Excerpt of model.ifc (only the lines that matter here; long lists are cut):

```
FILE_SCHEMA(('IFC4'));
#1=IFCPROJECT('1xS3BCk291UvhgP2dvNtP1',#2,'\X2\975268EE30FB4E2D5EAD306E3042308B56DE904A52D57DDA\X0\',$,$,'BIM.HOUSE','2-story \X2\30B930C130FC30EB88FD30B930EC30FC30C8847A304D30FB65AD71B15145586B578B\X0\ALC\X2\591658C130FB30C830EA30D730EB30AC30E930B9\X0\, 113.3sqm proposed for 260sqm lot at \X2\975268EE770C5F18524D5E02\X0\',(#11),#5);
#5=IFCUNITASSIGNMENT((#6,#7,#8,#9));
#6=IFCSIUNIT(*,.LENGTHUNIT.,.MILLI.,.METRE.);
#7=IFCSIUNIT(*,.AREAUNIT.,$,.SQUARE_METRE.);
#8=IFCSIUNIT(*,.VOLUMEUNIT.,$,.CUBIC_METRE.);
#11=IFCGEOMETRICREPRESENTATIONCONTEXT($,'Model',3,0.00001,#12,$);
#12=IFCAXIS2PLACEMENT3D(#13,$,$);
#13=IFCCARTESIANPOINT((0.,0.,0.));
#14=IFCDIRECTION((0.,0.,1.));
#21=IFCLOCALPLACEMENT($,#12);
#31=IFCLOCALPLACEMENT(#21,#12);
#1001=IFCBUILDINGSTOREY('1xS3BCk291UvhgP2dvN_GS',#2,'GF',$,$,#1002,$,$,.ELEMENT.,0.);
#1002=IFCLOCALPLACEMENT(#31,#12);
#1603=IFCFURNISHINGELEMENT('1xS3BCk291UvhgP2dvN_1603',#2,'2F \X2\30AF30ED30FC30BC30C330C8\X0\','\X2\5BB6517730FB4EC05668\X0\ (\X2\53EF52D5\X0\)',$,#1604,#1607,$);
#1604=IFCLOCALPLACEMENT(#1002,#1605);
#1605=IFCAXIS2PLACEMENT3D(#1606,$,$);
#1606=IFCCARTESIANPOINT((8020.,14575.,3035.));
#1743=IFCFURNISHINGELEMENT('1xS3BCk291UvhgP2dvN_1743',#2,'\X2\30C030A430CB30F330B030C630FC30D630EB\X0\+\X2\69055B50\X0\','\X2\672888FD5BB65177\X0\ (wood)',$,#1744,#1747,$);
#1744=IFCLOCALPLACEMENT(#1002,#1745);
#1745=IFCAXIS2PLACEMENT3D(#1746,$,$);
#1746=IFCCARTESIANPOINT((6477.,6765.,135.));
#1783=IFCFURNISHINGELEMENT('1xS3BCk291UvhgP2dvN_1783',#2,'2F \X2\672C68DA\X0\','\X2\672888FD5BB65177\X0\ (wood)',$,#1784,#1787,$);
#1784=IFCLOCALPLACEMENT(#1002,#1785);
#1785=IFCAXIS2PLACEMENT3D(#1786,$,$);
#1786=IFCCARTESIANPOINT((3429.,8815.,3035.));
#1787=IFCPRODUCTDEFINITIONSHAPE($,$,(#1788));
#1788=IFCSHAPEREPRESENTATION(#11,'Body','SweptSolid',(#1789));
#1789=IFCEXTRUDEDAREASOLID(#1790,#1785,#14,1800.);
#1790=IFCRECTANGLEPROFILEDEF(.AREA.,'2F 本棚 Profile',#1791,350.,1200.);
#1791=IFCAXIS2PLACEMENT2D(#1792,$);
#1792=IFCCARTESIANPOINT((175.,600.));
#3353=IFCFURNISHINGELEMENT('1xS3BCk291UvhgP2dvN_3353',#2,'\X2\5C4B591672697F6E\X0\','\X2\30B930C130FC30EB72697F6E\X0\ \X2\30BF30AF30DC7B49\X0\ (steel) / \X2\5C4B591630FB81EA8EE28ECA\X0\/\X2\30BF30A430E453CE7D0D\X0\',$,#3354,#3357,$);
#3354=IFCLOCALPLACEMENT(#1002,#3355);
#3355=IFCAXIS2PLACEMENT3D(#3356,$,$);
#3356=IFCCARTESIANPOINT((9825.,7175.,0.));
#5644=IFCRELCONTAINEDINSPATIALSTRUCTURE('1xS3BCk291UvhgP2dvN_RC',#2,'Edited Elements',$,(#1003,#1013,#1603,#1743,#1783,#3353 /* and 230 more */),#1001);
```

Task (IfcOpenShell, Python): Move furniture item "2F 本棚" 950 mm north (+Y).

```python
import ifcopenshell
import ifcopenshell.api.geometry
import ifcopenshell.util.placement

model = ifcopenshell.open("model.ifc")

item = model.by_guid("1xS3BCk291UvhgP2dvN_1783")
matrix = ifcopenshell.util.placement.get_local_placement(item.ObjectPlacement)
matrix[1, 3] += 950.0
ifcopenshell.api.geometry.edit_object_placement(model, product=item, matrix=matrix, is_si=False)

print(ifcopenshell.util.placement.get_local_placement(item.ObjectPlacement).round(3) + 0.0)

model.write("model_rev.ifc")
```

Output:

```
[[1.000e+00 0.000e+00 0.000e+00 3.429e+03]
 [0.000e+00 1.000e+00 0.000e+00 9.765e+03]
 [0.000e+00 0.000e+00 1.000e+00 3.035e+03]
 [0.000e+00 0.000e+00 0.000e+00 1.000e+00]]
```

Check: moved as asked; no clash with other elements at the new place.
